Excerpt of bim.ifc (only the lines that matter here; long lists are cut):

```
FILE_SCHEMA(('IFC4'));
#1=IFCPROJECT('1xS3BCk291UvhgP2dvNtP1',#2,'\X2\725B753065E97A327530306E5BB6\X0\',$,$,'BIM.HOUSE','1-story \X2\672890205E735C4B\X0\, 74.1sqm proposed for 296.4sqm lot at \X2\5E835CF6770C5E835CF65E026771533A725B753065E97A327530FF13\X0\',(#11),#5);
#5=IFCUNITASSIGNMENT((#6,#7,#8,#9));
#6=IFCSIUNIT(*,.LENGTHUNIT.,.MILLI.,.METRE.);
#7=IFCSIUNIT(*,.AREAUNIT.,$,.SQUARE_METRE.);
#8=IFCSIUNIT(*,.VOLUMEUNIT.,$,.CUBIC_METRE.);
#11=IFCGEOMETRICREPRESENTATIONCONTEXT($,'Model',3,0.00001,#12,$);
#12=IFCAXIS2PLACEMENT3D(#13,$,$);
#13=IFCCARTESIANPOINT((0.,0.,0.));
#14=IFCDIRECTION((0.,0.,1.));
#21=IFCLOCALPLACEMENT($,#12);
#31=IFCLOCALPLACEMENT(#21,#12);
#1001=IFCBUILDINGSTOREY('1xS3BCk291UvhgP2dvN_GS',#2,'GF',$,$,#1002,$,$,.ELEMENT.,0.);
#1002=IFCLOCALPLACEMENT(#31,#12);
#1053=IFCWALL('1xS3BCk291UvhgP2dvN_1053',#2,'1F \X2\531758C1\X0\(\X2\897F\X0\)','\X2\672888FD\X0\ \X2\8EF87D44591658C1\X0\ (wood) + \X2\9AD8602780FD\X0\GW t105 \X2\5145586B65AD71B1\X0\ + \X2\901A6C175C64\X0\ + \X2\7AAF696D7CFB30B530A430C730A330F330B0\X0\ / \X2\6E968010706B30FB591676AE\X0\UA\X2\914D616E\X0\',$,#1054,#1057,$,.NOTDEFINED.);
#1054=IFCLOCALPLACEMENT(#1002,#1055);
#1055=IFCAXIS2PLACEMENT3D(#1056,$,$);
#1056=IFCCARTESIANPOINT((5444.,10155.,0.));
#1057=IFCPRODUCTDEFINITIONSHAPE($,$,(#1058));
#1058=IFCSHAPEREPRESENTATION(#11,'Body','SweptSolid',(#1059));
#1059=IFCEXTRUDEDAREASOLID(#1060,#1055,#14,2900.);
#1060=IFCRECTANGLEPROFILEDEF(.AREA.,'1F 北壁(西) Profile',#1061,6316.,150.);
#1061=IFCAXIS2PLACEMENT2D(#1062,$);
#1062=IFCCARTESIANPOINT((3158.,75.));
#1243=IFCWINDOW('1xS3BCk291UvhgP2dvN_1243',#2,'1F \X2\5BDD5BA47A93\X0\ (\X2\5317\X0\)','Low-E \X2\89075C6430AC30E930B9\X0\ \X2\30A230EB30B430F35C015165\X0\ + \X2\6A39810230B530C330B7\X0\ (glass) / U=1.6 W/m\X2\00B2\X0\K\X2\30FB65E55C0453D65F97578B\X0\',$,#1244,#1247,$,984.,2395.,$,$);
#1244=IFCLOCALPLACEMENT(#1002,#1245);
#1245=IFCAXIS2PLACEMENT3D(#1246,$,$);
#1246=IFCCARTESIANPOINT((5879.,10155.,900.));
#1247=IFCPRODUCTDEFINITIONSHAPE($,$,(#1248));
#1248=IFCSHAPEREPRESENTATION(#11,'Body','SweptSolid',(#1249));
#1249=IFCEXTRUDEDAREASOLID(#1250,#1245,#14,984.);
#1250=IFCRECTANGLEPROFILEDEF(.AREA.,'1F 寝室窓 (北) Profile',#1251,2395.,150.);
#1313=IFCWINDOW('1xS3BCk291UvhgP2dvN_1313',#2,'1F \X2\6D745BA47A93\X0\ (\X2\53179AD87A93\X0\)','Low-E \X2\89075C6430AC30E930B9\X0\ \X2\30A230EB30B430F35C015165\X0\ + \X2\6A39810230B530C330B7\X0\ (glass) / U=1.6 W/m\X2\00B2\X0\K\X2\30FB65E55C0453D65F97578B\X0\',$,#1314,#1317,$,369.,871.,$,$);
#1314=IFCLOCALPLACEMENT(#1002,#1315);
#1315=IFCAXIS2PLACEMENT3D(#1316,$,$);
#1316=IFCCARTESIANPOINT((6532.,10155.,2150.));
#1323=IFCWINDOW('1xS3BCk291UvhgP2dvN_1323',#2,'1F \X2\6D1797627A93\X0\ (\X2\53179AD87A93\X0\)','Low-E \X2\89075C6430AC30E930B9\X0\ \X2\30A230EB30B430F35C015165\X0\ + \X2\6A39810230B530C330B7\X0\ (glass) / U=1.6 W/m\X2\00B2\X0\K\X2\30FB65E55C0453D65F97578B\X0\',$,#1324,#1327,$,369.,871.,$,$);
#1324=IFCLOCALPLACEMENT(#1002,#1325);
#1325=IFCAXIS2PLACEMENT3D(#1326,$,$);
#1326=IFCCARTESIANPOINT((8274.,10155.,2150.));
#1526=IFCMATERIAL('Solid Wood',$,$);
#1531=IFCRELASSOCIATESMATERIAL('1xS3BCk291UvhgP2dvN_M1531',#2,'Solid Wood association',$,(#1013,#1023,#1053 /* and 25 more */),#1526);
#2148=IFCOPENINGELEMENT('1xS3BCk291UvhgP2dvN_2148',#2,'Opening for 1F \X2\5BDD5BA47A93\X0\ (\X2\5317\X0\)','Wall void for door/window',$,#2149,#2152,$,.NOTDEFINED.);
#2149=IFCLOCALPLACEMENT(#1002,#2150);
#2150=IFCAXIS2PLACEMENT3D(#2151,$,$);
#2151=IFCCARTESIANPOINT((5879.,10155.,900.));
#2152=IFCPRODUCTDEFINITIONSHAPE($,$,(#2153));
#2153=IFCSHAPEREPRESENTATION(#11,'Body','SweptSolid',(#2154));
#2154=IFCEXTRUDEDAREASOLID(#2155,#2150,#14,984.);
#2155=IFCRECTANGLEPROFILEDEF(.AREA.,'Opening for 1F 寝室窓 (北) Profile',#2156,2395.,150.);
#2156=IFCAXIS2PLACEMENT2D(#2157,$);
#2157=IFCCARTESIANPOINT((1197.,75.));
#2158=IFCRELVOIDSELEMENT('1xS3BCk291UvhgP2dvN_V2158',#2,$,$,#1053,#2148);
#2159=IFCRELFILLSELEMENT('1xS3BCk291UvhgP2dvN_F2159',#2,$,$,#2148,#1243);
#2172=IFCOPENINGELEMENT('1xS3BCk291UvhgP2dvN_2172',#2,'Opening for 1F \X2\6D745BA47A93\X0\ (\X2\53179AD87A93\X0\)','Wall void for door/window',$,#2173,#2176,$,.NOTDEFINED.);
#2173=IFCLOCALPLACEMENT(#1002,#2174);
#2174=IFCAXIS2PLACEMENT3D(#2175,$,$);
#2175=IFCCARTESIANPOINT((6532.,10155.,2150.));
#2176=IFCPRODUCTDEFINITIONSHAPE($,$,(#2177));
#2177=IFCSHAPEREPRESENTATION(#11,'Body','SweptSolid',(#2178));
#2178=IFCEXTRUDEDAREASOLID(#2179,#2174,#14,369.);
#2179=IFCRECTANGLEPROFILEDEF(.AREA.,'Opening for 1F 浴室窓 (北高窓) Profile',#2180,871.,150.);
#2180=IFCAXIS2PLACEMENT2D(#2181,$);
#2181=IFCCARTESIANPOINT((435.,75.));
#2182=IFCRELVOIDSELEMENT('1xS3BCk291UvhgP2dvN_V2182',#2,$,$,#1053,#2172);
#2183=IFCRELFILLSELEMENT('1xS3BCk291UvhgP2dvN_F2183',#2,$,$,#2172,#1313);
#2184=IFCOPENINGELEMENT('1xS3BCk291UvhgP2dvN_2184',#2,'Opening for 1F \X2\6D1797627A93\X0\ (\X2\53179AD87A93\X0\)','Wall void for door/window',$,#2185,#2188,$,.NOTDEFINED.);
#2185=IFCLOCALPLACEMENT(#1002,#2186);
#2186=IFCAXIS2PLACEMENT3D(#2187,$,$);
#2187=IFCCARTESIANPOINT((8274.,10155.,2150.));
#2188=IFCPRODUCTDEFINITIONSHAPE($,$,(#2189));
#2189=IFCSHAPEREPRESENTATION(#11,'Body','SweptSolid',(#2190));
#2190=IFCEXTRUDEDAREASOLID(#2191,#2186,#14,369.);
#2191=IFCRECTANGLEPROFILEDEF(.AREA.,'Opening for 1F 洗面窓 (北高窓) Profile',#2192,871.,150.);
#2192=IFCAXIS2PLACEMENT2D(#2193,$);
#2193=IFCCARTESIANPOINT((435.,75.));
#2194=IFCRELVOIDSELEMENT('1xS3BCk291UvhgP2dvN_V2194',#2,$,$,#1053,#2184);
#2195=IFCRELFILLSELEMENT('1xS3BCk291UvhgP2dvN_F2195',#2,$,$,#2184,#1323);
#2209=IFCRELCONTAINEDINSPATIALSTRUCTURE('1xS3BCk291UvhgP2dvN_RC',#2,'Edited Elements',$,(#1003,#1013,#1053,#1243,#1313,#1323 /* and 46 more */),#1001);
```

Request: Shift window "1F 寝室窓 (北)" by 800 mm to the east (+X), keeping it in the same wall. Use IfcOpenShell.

```python
import ifcopenshell
import ifcopenshell.api.geometry
import ifcopenshell.util.placement

model = ifcopenshell.open("bim.ifc")

window = model.by_id(1243)
opening = window.FillsVoids[0].RelatingOpeningElement
wall = opening.VoidsElements[0].RelatingBuildingElement

wall_matrix = ifcopenshell.util.placement.get_local_placement(wall.ObjectPlacement)
shift = wall_matrix[:3, 0] * 800.0
before = ifcopenshell.util.placement.get_local_placement(window.ObjectPlacement)[:3, 3].copy()

# The window is not placed relative to its opening, so move both.
for product in (opening, window):
    matrix = ifcopenshell.util.placement.get_local_placement(product.ObjectPlacement)
    matrix[:3, 3] += shift
    ifcopenshell.api.geometry.edit_object_placement(model, product=product, matrix=matrix, is_si=False)

after = ifcopenshell.util.placement.get_local_placement(window.ObjectPlacement)[:3, 3]
print("window moved by", (after - before).round(3) + 0.0)

model.write("bim_updated.ifc")
```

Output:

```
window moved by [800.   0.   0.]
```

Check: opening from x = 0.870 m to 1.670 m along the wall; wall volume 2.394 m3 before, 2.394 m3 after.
